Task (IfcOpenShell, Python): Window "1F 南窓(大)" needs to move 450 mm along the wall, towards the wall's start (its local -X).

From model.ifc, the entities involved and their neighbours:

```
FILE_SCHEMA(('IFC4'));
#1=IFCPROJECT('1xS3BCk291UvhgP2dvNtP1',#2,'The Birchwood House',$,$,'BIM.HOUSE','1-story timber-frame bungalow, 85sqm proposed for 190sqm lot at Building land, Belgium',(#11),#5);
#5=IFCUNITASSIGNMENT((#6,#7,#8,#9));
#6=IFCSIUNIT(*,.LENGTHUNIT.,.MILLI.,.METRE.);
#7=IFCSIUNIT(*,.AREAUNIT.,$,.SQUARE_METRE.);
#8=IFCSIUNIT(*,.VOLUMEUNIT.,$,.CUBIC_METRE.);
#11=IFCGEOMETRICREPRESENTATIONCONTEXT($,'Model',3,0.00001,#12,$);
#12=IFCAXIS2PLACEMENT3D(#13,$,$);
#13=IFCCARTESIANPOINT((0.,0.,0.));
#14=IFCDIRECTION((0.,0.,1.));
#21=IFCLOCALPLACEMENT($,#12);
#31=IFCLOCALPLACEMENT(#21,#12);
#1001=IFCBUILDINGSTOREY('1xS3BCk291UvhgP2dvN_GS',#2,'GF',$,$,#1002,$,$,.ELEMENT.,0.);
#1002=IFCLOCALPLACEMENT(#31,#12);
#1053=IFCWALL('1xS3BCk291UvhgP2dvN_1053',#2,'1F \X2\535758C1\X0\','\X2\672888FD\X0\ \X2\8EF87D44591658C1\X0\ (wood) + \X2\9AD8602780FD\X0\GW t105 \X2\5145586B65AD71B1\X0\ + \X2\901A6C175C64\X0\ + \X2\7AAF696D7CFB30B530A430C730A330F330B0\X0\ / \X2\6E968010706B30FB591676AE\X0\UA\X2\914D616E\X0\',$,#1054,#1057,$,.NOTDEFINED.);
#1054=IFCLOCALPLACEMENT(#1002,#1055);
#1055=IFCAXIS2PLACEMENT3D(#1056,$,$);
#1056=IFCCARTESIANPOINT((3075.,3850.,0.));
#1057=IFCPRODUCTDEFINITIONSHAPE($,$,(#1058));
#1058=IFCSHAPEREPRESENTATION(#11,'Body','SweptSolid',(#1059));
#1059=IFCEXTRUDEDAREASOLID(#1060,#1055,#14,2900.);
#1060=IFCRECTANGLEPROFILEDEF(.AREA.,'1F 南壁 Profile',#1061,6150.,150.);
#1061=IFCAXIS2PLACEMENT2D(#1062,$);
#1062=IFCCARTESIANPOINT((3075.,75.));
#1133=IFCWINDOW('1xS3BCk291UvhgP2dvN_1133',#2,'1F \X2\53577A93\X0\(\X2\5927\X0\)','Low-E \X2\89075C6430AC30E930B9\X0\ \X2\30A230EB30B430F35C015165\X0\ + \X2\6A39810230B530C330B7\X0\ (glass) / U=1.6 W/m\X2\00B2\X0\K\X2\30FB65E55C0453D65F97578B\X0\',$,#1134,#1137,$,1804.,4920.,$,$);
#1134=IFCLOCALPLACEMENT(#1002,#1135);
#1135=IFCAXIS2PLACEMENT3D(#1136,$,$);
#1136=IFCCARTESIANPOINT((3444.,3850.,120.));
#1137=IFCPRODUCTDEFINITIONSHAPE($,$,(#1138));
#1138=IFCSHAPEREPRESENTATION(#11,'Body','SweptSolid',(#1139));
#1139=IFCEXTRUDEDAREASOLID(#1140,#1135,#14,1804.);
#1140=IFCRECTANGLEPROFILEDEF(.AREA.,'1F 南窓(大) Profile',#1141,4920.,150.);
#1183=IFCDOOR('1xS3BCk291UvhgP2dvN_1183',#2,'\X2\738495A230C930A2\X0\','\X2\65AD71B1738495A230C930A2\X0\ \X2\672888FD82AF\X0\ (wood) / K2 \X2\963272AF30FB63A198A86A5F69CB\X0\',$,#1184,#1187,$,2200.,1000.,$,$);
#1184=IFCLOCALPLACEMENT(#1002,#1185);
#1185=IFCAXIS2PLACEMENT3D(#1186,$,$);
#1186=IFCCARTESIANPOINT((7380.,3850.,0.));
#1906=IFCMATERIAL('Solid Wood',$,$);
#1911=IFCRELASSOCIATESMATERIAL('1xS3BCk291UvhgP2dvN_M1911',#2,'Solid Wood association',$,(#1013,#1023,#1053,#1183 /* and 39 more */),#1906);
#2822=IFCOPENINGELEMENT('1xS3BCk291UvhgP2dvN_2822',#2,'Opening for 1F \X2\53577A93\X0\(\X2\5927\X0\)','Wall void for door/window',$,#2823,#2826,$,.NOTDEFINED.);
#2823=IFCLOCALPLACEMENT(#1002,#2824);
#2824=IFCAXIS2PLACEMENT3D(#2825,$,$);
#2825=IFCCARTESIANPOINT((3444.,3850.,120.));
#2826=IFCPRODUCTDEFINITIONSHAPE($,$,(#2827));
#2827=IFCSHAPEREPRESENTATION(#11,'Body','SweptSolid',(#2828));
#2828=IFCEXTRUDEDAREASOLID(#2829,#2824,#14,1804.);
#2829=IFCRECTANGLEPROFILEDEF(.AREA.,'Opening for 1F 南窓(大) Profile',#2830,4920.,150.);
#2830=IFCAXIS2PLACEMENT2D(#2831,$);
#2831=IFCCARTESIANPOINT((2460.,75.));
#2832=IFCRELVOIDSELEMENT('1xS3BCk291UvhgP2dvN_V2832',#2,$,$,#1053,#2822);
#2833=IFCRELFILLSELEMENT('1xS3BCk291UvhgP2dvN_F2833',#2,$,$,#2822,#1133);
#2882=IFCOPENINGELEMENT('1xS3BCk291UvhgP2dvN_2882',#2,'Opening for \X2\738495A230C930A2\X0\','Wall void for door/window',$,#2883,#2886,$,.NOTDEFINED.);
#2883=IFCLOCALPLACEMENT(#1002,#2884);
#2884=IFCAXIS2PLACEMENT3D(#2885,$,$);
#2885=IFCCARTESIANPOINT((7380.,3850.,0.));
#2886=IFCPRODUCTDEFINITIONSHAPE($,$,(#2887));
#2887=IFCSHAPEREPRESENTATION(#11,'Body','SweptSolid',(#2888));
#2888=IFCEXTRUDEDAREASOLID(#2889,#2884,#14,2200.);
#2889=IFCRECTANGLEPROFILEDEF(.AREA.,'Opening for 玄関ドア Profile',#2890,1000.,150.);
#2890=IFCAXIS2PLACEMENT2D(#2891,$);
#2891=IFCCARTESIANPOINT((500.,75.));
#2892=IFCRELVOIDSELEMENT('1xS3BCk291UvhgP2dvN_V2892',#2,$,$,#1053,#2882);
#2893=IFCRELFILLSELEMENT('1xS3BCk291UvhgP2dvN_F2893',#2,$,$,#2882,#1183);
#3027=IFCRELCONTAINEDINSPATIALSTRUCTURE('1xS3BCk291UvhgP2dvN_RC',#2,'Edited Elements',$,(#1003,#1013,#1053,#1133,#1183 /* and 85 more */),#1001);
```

```python
import ifcopenshell
import ifcopenshell.api.geometry
import ifcopenshell.util.placement
import ifcopenshell.util.unit

model = ifcopenshell.open("model.ifc")
unit_scale = ifcopenshell.util.unit.calculate_unit_scale(model)

window = model.by_guid("1xS3BCk291UvhgP2dvN_1133")
opening = window.FillsVoids[0].RelatingOpeningElement
wall = opening.VoidsElements[0].RelatingBuildingElement

wall_matrix = ifcopenshell.util.placement.get_local_placement(wall.ObjectPlacement)
shift = wall_matrix[:3, 0] * -0.45 / unit_scale
before = ifcopenshell.util.placement.get_local_placement(window.ObjectPlacement)[:3, 3].copy()

# The window is not placed relative to its opening, so move both.
for product in (opening, window):
    matrix = ifcopenshell.util.placement.get_local_placement(product.ObjectPlacement)
    matrix[:3, 3] += shift
    ifcopenshell.api.geometry.edit_object_placement(model, product=product, matrix=matrix, is_si=False)

after = ifcopenshell.util.placement.get_local_placement(window.ObjectPlacement)[:3, 3]
print("window moved by", (after - before).round(3) + 0.0)

model.write("model_updated.ifc")
```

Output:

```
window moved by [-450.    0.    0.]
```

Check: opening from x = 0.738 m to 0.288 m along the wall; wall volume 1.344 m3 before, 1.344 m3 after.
